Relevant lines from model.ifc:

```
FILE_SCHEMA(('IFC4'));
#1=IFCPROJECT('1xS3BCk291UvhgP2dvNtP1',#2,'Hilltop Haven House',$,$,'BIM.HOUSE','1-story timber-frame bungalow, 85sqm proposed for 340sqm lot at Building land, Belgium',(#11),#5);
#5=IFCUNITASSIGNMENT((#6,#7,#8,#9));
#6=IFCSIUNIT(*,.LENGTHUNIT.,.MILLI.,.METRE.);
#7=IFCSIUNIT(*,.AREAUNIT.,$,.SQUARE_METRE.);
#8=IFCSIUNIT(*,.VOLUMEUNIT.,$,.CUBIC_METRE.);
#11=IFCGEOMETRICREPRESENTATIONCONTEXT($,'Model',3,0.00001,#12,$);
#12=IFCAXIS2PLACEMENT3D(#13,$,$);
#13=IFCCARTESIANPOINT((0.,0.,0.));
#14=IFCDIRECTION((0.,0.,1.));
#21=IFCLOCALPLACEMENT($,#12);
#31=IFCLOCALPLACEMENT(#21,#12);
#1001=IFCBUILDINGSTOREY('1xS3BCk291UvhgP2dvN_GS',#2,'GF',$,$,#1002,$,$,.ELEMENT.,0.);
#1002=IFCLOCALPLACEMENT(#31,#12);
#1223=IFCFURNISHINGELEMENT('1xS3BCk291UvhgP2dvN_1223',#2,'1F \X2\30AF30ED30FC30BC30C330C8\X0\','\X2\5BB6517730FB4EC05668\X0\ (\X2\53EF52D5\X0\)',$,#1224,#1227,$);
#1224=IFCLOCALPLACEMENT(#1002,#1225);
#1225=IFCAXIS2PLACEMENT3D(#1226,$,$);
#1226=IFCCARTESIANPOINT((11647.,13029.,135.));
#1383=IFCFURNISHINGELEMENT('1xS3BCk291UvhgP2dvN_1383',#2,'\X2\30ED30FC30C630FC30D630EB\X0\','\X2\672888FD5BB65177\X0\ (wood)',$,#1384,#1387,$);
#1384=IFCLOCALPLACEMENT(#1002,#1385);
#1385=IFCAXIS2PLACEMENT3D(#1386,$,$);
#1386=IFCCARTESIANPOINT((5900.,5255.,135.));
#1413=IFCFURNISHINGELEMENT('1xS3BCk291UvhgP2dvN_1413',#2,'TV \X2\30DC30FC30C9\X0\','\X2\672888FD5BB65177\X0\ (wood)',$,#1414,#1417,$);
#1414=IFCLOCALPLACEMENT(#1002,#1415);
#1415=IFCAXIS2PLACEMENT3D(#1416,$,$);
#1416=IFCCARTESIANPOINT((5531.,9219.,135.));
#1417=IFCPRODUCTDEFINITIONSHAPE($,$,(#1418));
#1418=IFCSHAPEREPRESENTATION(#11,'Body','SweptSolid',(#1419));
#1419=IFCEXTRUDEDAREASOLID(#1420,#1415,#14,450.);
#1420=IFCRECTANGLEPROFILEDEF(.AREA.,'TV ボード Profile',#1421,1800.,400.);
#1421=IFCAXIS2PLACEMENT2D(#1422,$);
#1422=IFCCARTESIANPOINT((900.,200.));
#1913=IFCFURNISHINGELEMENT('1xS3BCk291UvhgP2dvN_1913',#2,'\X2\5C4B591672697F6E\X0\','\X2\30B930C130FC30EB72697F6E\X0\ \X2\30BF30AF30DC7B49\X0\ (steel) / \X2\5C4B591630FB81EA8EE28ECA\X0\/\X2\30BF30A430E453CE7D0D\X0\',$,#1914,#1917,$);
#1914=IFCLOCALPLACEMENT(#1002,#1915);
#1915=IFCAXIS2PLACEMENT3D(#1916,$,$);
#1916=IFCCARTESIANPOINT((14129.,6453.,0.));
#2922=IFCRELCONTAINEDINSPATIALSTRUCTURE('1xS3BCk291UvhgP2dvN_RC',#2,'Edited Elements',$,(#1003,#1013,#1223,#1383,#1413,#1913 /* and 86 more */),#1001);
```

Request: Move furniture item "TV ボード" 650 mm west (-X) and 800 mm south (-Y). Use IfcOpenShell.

```python
import ifcopenshell
import ifcopenshell.api.geometry
import ifcopenshell.util.placement
import ifcopenshell.util.unit

model = ifcopenshell.open("model.ifc")
unit_scale = ifcopenshell.util.unit.calculate_unit_scale(model)

item = model.by_guid("1xS3BCk291UvhgP2dvN_1413")
matrix = ifcopenshell.util.placement.get_local_placement(item.ObjectPlacement)
matrix[0, 3] -= 0.65 / unit_scale
matrix[1, 3] -= 0.8 / unit_scale
ifcopenshell.api.geometry.edit_object_placement(model, product=item, matrix=matrix, is_si=False)

print(ifcopenshell.util.placement.get_local_placement(item.ObjectPlacement).round(3) + 0.0)

model.write("model_rev.ifc")
```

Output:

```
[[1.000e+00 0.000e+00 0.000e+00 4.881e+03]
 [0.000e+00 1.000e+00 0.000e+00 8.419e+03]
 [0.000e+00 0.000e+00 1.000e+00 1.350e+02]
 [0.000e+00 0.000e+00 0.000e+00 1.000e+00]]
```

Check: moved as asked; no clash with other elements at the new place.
